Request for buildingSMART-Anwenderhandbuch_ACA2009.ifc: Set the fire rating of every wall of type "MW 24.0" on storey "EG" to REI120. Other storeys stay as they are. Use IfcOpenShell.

First a look at what the model holds.

```python
import ifcopenshell
import ifcopenshell.util.element

model = ifcopenshell.open("buildingSMART-Anwenderhandbuch_ACA2009.ifc")
print(model.schema)
storey = next(s for s in model.by_type("IfcBuildingStorey") if s.Name == "EG")
walls = [e for e in ifcopenshell.util.element.get_decomposition(storey) if e.is_a("IfcWall")]
seen = {}
for e in walls:
    element_type = ifcopenshell.util.element.get_type(e)
    key = (element_type.Name if element_type != e and element_type else None, ifcopenshell.util.element.get_pset(e, "Pset_WallCommon", "FireRating"))
    seen[key] = seen.get(key, 0) + 1
for (name, value), count in sorted(seen.items(), key=str):
    print(count, "x", name, "|", value)
```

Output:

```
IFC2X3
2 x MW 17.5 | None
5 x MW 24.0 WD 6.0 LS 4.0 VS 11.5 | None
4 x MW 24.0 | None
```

```python
import ifcopenshell
import ifcopenshell.api.pset
import ifcopenshell.util.element

model = ifcopenshell.open("buildingSMART-Anwenderhandbuch_ACA2009.ifc")

storey = next(s for s in model.by_type("IfcBuildingStorey") if s.Name == "EG")
walls = [e for e in ifcopenshell.util.element.get_decomposition(storey) if e.is_a("IfcWall")]

count = 0
for e in walls:
    element_type = ifcopenshell.util.element.get_type(e)
    if element_type in (None, e) or element_type.Name != "MW 24.0":
        continue
    # add_pset returns the element's existing set when there is one.
    pset = ifcopenshell.api.pset.add_pset(model, product=e, name="Pset_WallCommon")
    ifcopenshell.api.pset.edit_pset(model, pset=pset, properties={"FireRating": "REI120"})
    count += 1

print(count, "walls updated")

model.write("buildingSMART-Anwenderhandbuch_ACA2009_edited.ifc")
```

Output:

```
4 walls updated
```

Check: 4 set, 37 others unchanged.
